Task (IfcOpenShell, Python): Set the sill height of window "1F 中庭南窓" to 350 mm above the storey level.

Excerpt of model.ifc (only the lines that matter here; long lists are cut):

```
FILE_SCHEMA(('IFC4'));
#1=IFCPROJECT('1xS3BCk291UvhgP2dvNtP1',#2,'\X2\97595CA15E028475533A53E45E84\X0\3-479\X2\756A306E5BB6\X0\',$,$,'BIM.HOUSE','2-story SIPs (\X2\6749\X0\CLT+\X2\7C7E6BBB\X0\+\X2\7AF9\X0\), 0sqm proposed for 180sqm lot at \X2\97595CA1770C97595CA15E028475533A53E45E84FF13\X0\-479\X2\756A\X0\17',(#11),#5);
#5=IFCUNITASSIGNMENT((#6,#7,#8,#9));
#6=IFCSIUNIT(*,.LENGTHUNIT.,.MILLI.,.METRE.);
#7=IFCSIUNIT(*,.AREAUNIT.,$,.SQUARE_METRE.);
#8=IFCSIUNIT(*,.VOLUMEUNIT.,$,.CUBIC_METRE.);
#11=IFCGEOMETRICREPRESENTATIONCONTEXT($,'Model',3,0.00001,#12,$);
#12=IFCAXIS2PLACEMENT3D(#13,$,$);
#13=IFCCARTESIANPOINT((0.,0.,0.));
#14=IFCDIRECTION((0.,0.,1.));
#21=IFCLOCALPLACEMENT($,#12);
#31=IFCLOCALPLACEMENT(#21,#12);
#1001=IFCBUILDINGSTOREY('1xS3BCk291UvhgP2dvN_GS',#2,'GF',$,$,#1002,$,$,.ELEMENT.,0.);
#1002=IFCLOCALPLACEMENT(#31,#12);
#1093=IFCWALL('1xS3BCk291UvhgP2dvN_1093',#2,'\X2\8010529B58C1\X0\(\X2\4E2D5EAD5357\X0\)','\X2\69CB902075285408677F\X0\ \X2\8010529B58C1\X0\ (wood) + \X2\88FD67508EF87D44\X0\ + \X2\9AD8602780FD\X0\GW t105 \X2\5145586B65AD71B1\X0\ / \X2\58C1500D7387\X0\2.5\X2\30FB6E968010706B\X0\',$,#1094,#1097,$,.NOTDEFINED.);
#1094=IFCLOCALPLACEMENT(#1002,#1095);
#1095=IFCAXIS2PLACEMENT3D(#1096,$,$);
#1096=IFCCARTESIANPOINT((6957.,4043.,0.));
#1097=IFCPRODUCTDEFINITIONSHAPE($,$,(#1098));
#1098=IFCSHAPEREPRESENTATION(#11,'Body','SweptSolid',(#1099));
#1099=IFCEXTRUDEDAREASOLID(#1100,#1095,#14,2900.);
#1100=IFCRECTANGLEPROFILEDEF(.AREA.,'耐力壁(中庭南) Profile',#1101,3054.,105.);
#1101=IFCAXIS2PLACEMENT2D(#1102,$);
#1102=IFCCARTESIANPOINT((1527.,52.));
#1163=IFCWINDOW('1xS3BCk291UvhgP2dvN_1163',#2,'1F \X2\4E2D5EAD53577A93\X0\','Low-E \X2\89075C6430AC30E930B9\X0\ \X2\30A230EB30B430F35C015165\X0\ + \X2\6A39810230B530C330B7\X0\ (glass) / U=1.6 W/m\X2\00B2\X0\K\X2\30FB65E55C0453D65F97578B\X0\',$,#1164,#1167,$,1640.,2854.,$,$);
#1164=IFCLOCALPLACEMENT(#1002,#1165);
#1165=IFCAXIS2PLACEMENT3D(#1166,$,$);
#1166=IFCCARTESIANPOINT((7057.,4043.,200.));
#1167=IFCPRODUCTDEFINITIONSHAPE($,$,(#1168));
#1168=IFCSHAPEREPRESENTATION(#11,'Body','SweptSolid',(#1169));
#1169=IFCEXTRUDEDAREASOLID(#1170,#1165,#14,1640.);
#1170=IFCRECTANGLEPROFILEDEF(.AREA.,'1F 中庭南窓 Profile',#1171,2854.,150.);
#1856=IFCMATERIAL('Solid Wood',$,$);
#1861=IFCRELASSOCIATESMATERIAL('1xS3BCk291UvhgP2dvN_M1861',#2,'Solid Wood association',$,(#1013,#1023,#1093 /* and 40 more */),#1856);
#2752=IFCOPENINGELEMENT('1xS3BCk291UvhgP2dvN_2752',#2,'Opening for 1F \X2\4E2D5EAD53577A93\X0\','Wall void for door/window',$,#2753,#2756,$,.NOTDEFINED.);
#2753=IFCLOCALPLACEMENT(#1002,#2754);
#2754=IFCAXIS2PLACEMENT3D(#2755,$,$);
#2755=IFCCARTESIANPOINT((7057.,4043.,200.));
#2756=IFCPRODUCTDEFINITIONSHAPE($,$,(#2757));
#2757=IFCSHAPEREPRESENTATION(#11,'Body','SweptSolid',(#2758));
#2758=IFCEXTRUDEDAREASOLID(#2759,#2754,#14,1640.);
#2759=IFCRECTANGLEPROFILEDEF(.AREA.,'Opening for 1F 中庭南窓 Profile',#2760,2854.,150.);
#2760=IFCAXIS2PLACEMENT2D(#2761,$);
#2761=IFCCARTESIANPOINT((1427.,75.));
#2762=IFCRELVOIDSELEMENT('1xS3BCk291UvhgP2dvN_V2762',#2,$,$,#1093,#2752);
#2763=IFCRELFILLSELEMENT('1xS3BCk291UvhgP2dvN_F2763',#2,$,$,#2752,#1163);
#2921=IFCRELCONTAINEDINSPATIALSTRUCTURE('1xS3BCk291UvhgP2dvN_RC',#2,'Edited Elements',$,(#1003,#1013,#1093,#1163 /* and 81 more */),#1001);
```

```python
import numpy as np
import ifcopenshell
import ifcopenshell.api.geometry
import ifcopenshell.geom
import ifcopenshell.util.element
import ifcopenshell.util.placement
import ifcopenshell.util.shape
import ifcopenshell.util.unit

model = ifcopenshell.open("model.ifc")
unit_scale = ifcopenshell.util.unit.calculate_unit_scale(model)

window = model.by_guid("1xS3BCk291UvhgP2dvN_1163")
opening = window.FillsVoids[0].RelatingOpeningElement
storey = ifcopenshell.util.element.get_container(window, ifc_class="IfcBuildingStorey")
level = ifcopenshell.util.placement.get_local_placement(storey.ObjectPlacement)[2, 3]

# The opening's origin need not be at the sill, so measure its lowest point.
shape = ifcopenshell.geom.create_shape(ifcopenshell.geom.settings(), opening)
bottom = ifcopenshell.util.shape.get_shape_bottom_elevation(shape, shape.geometry) / unit_scale
dz = level + 350.0 - bottom

shift = np.array([0.0, 0.0, dz])
# The window is not placed relative to its opening, so move both.
for product in (opening, window):
    matrix = ifcopenshell.util.placement.get_local_placement(product.ObjectPlacement)
    matrix[:3, 3] += shift
    ifcopenshell.api.geometry.edit_object_placement(model, product=product, matrix=matrix, is_si=False)

print(f"moved by {dz * unit_scale:+.3f} m")

model.write("model_v2.ifc")
```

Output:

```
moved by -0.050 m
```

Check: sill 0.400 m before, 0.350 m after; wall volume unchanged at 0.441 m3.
